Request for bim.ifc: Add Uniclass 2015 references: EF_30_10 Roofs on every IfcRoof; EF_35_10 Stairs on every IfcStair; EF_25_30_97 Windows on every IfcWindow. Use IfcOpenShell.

First a look at what the model holds.

```python
import ifcopenshell

model = ifcopenshell.open("bim.ifc")
print(model.schema)
print("classifications:", [c.Name for c in model.by_type("IfcClassification")])
for ifc_class in ("IfcDoor", "IfcRoof", "IfcStair", "IfcWall", "IfcWindow"):
    print(ifc_class, len(model.by_type(ifc_class)))
```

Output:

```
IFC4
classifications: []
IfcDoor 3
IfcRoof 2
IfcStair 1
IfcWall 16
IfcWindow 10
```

```python
import ifcopenshell
import ifcopenshell.api.classification

model = ifcopenshell.open("bim.ifc")

system = ifcopenshell.api.classification.add_classification(model, classification="Uniclass 2015")

codes = {
    "IfcRoof": ("EF_30_10", "Roofs"),
    "IfcStair": ("EF_35_10", "Stairs"),
    "IfcWindow": ("EF_25_30_97", "Windows"),
}
for ifc_class, (code, name) in codes.items():
    products = model.by_type(ifc_class)
    ifcopenshell.api.classification.add_reference(
        model, products=products, classification=system, identification=code, name=name
    )
    print(code, len(products))

model.write("bim-out.ifc")
```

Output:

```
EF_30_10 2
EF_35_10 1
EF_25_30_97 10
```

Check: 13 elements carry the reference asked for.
